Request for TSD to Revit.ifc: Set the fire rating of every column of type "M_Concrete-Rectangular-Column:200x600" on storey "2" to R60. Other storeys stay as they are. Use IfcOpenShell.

First a look at what the model holds.

```python
import ifcopenshell
import ifcopenshell.util.element

model = ifcopenshell.open("TSD to Revit.ifc")
print(model.schema)
storey = next(s for s in model.by_type("IfcBuildingStorey") if s.Name == "2")
columns = [e for e in ifcopenshell.util.element.get_decomposition(storey) if e.is_a("IfcColumn")]
seen = {}
for e in columns:
    element_type = ifcopenshell.util.element.get_type(e)
    key = (element_type.Name if element_type != e and element_type else None, ifcopenshell.util.element.get_pset(e, "Pset_ColumnCommon", "FireRating"))
    seen[key] = seen.get(key, 0) + 1
for (name, value), count in sorted(seen.items(), key=str):
    print(count, "x", name, "|", value)
```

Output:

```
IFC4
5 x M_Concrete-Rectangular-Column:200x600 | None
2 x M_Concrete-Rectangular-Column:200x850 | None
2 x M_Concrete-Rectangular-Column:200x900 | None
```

```python
import ifcopenshell
import ifcopenshell.api.pset
import ifcopenshell.util.element

model = ifcopenshell.open("TSD to Revit.ifc")

storey = next(s for s in model.by_type("IfcBuildingStorey") if s.Name == "2")
columns = [e for e in ifcopenshell.util.element.get_decomposition(storey) if e.is_a("IfcColumn")]

count = 0
for e in columns:
    element_type = ifcopenshell.util.element.get_type(e)
    if element_type in (None, e) or element_type.Name != "M_Concrete-Rectangular-Column:200x600":
        continue
    # add_pset returns the element's existing set when there is one.
    pset = ifcopenshell.api.pset.add_pset(model, product=e, name="Pset_ColumnCommon")
    ifcopenshell.api.pset.edit_pset(model, pset=pset, properties={"FireRating": "R60"})
    count += 1

print(count, "columns updated")

model.write("TSD to Revit_edited.ifc")
```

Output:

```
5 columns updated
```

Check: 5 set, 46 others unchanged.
